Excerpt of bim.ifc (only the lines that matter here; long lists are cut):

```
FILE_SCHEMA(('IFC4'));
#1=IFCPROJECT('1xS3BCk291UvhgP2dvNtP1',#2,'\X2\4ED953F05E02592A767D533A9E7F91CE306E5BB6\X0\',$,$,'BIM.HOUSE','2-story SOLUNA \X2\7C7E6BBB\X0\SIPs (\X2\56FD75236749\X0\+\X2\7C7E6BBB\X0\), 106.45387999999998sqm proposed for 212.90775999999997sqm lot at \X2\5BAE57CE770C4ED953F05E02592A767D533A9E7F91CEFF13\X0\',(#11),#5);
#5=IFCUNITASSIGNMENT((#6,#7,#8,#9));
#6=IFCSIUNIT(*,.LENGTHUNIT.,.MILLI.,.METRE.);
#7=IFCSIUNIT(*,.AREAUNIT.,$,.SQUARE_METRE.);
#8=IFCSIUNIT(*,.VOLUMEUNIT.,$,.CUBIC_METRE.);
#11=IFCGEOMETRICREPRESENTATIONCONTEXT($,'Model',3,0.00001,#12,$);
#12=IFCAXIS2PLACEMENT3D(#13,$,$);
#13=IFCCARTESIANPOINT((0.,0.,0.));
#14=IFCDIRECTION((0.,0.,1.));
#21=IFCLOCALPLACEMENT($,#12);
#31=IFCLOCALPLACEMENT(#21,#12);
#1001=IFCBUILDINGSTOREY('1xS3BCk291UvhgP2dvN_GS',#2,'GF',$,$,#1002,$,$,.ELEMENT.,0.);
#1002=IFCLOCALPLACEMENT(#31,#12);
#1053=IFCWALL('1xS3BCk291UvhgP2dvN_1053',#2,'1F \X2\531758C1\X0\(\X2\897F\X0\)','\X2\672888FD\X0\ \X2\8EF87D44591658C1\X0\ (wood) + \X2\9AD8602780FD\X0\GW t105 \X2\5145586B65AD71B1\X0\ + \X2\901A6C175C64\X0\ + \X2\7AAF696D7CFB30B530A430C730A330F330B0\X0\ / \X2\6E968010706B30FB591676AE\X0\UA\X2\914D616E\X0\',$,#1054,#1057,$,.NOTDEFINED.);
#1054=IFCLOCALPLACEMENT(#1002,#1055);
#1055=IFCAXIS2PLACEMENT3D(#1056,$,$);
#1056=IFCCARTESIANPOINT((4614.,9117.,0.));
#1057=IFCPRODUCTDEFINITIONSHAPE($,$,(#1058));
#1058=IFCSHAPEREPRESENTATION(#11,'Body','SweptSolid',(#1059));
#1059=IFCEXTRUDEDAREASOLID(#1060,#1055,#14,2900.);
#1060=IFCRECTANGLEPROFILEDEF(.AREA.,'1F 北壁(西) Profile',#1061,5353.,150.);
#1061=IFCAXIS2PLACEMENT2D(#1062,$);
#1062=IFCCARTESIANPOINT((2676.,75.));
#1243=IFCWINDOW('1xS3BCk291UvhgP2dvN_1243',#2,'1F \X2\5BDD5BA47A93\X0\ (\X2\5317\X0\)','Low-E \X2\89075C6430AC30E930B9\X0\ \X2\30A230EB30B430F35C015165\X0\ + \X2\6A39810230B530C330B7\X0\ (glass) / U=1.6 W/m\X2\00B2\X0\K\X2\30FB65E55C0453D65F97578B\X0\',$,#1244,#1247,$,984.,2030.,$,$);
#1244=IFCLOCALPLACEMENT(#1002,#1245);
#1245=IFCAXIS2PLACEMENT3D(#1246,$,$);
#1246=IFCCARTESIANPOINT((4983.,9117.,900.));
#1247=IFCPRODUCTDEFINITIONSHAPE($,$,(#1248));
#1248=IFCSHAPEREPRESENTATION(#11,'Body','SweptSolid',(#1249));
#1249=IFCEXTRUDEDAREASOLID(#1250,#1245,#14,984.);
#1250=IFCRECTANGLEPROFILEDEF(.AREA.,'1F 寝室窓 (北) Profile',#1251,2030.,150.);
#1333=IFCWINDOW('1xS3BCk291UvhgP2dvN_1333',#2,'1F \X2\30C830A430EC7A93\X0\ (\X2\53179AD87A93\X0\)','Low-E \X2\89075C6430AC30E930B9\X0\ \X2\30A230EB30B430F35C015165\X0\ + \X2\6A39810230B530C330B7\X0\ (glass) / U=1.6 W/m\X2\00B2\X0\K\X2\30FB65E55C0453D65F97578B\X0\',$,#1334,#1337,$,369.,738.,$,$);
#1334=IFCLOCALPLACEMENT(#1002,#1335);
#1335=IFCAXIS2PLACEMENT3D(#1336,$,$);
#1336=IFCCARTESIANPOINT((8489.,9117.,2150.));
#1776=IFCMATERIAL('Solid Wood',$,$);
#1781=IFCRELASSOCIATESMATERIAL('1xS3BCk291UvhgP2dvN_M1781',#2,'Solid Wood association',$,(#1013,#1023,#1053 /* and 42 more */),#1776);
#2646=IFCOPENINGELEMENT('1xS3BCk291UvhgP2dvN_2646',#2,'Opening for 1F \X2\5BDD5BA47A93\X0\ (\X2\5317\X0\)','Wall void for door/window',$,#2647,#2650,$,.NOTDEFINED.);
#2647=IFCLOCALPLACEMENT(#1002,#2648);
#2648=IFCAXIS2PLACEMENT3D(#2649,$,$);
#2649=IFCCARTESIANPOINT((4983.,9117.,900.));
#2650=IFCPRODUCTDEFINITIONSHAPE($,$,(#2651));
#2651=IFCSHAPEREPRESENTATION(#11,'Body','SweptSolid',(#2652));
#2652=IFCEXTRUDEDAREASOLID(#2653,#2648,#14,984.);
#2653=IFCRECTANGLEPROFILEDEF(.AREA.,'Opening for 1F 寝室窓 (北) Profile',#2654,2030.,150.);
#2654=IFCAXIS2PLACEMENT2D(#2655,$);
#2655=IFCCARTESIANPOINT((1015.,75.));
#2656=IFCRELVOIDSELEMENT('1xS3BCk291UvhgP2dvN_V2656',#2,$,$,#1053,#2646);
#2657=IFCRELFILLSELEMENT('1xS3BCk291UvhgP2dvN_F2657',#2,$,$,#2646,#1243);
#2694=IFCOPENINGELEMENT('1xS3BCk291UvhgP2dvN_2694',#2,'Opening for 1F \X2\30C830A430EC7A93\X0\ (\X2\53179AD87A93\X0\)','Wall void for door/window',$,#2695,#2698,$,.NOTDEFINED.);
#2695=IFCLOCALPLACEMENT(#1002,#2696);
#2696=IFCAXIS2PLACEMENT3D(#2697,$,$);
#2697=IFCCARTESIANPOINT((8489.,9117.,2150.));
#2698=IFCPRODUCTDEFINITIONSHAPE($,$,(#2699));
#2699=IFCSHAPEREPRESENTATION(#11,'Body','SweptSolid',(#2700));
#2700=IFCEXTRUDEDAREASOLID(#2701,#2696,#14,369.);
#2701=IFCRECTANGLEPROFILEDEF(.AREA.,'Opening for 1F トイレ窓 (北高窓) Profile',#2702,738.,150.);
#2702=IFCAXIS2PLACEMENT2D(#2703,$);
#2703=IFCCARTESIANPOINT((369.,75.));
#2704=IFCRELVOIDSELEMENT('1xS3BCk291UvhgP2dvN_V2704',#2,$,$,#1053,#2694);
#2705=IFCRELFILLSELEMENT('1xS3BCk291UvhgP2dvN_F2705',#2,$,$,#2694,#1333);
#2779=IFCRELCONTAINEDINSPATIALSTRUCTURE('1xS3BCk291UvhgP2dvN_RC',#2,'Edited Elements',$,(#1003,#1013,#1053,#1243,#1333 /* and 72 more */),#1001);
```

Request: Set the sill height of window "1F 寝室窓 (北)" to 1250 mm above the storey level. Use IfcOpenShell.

```python
import numpy as np
import ifcopenshell
import ifcopenshell.api.geometry
import ifcopenshell.geom
import ifcopenshell.util.element
import ifcopenshell.util.placement
import ifcopenshell.util.shape
import ifcopenshell.util.unit

model = ifcopenshell.open("bim.ifc")
unit_scale = ifcopenshell.util.unit.calculate_unit_scale(model)

window = model.by_id(1243)
opening = window.FillsVoids[0].RelatingOpeningElement
storey = ifcopenshell.util.element.get_container(window, ifc_class="IfcBuildingStorey")
level = ifcopenshell.util.placement.get_local_placement(storey.ObjectPlacement)[2, 3]

# The opening's origin need not be at the sill, so measure its lowest point.
shape = ifcopenshell.geom.create_shape(ifcopenshell.geom.settings(), opening)
bottom = ifcopenshell.util.shape.get_shape_bottom_elevation(shape, shape.geometry) / unit_scale
dz = level + 1250.0 - bottom

shift = np.array([0.0, 0.0, dz])
# The window is not placed relative to its opening, so move both.
for product in (opening, window):
    matrix = ifcopenshell.util.placement.get_local_placement(product.ObjectPlacement)
    matrix[:3, 3] += shift
    ifcopenshell.api.geometry.edit_object_placement(model, product=product, matrix=matrix, is_si=False)

print(f"moved by {dz * unit_scale:+.3f} m")

model.write("bim_updated.ifc")
```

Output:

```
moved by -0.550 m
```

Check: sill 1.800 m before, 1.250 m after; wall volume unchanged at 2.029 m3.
